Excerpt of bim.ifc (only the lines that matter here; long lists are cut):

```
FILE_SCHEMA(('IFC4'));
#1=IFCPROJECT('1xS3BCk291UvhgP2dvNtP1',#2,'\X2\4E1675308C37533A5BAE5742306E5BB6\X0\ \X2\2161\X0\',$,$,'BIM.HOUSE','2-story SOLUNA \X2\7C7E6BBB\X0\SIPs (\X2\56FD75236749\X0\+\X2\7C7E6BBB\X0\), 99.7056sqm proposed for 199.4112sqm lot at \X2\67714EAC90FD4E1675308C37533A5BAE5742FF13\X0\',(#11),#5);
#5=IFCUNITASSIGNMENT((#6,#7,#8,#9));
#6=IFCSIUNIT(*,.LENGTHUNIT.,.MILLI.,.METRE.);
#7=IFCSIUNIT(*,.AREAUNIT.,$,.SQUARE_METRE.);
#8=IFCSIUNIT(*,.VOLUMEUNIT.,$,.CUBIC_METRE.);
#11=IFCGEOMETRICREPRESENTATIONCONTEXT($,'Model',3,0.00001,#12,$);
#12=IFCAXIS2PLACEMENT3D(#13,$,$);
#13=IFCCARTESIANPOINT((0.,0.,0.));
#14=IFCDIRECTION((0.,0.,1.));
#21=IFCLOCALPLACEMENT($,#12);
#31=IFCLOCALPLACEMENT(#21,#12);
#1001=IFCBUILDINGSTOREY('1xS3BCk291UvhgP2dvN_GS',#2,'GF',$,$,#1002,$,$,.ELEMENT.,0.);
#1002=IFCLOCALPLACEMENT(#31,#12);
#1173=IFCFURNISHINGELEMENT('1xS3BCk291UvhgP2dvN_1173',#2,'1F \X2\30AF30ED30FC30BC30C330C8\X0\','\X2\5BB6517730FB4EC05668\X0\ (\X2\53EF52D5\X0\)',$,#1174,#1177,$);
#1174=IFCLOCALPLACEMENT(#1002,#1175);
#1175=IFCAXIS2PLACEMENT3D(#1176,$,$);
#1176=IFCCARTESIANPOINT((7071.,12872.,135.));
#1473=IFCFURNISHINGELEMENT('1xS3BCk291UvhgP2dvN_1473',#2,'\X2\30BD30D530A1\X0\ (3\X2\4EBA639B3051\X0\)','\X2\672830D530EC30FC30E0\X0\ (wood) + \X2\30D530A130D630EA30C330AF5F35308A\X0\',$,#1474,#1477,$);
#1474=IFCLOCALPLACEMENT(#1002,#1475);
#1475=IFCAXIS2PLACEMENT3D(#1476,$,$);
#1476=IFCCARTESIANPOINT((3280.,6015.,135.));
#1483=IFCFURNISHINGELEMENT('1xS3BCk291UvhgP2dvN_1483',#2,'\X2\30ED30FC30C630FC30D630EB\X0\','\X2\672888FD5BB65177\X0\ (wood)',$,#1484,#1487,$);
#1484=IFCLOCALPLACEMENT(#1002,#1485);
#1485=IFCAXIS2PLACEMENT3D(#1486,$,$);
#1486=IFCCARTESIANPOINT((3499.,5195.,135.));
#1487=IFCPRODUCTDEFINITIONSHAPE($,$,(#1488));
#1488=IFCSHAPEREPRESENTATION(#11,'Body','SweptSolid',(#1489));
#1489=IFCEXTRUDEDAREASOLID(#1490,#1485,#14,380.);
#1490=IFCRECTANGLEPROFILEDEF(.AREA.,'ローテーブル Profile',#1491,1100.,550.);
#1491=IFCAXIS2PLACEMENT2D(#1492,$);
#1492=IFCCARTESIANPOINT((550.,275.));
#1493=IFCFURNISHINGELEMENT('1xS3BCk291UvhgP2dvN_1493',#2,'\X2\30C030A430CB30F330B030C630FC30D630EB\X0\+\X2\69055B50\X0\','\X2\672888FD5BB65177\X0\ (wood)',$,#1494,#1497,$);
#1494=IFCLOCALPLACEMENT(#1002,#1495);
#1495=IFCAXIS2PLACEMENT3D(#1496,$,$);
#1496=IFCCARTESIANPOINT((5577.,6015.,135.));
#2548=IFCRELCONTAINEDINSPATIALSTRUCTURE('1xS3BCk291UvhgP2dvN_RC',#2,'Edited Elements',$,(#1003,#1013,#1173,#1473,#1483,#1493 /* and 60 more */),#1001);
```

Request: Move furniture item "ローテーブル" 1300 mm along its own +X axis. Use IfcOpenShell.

```python
import ifcopenshell
import ifcopenshell.api.geometry
import ifcopenshell.util.placement

model = ifcopenshell.open("bim.ifc")

item = model.by_id(1483)
matrix = ifcopenshell.util.placement.get_local_placement(item.ObjectPlacement)
matrix[:3, 3] += matrix[:3, 0] * 1300.0
ifcopenshell.api.geometry.edit_object_placement(model, product=item, matrix=matrix, is_si=False)

print(ifcopenshell.util.placement.get_local_placement(item.ObjectPlacement).round(3) + 0.0)

model.write("bim_rev.ifc")
```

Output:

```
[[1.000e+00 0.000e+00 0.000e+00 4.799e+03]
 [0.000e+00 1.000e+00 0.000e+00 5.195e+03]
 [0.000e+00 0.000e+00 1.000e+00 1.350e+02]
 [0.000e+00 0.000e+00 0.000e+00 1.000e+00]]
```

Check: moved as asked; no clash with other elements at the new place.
